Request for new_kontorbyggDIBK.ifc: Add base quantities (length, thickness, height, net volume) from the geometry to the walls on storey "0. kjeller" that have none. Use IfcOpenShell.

First a look at what the model holds.

```python
import ifcopenshell
import ifcopenshell.util.element
import ifcopenshell.util.unit

model = ifcopenshell.open("new_kontorbyggDIBK.ifc")
print(model.schema)
for unit_type in ("LENGTHUNIT", "AREAUNIT", "VOLUMEUNIT"):
    print(unit_type, ifcopenshell.util.unit.calculate_unit_scale(model, unit_type))
storey = next(s for s in model.by_type("IfcBuildingStorey") if s.Name == "0. kjeller")
walls = [e for e in ifcopenshell.util.element.get_decomposition(storey) if e.is_a("IfcWall")]
for e in sorted(walls, key=lambda e: e.id()):
    print(e.id(), e.is_a(), e.Name, list(ifcopenshell.util.element.get_psets(e, qtos_only=True)), sep=" | ")
```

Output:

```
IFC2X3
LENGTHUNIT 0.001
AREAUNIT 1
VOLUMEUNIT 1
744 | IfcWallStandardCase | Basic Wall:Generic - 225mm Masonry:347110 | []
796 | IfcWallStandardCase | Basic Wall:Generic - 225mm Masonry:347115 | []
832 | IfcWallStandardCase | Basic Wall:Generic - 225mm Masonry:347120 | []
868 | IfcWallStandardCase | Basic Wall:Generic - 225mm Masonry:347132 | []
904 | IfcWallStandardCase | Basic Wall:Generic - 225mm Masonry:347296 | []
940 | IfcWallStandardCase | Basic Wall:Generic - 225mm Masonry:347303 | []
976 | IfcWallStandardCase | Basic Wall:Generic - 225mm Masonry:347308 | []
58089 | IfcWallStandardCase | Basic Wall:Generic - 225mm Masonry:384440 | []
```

```python
import ifcopenshell
import ifcopenshell.api.pset
import ifcopenshell.geom
import ifcopenshell.util.element
import ifcopenshell.util.shape
import ifcopenshell.util.unit

model = ifcopenshell.open("new_kontorbyggDIBK.ifc")
unit_scale = ifcopenshell.util.unit.calculate_unit_scale(model)
volume_scale = ifcopenshell.util.unit.calculate_unit_scale(model, "VOLUMEUNIT")
settings = ifcopenshell.geom.settings()

storey = next(s for s in model.by_type("IfcBuildingStorey") if s.Name == "0. kjeller")
walls = [e for e in ifcopenshell.util.element.get_decomposition(storey) if e.is_a("IfcWall")]

for e in sorted(walls, key=lambda e: e.id()):
    if ifcopenshell.util.element.get_psets(e, qtos_only=True, should_inherit=False):
        continue
    # Geometry comes back in metres, in the element's own axes.
    shape = ifcopenshell.geom.create_shape(settings, e)
    values = {
        "Length": ifcopenshell.util.shape.get_x(shape.geometry) / unit_scale,
        "Width": ifcopenshell.util.shape.get_y(shape.geometry) / unit_scale,
        "Height": ifcopenshell.util.shape.get_z(shape.geometry) / unit_scale,
        "NetVolume": ifcopenshell.util.shape.get_volume(shape.geometry) / volume_scale,
    }
    qto = ifcopenshell.api.pset.add_qto(model, product=e, name="BaseQuantities")
    ifcopenshell.api.pset.edit_qto(model, qto=qto, properties=values)
    print(e.id(), {k: round(v, 3) for k, v in values.items()})

model.write("new_kontorbyggDIBK_v2.ifc")
```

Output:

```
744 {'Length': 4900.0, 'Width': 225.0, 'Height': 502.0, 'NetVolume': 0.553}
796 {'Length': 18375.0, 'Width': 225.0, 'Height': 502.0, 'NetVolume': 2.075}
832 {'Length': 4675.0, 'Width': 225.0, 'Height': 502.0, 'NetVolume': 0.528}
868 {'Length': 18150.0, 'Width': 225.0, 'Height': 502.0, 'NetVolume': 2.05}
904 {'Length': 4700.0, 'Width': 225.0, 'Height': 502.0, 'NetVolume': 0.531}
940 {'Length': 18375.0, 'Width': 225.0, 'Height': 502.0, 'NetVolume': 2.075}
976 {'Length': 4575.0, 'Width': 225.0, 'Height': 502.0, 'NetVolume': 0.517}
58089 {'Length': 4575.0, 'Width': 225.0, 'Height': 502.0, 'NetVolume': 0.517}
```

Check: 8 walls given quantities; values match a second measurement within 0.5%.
